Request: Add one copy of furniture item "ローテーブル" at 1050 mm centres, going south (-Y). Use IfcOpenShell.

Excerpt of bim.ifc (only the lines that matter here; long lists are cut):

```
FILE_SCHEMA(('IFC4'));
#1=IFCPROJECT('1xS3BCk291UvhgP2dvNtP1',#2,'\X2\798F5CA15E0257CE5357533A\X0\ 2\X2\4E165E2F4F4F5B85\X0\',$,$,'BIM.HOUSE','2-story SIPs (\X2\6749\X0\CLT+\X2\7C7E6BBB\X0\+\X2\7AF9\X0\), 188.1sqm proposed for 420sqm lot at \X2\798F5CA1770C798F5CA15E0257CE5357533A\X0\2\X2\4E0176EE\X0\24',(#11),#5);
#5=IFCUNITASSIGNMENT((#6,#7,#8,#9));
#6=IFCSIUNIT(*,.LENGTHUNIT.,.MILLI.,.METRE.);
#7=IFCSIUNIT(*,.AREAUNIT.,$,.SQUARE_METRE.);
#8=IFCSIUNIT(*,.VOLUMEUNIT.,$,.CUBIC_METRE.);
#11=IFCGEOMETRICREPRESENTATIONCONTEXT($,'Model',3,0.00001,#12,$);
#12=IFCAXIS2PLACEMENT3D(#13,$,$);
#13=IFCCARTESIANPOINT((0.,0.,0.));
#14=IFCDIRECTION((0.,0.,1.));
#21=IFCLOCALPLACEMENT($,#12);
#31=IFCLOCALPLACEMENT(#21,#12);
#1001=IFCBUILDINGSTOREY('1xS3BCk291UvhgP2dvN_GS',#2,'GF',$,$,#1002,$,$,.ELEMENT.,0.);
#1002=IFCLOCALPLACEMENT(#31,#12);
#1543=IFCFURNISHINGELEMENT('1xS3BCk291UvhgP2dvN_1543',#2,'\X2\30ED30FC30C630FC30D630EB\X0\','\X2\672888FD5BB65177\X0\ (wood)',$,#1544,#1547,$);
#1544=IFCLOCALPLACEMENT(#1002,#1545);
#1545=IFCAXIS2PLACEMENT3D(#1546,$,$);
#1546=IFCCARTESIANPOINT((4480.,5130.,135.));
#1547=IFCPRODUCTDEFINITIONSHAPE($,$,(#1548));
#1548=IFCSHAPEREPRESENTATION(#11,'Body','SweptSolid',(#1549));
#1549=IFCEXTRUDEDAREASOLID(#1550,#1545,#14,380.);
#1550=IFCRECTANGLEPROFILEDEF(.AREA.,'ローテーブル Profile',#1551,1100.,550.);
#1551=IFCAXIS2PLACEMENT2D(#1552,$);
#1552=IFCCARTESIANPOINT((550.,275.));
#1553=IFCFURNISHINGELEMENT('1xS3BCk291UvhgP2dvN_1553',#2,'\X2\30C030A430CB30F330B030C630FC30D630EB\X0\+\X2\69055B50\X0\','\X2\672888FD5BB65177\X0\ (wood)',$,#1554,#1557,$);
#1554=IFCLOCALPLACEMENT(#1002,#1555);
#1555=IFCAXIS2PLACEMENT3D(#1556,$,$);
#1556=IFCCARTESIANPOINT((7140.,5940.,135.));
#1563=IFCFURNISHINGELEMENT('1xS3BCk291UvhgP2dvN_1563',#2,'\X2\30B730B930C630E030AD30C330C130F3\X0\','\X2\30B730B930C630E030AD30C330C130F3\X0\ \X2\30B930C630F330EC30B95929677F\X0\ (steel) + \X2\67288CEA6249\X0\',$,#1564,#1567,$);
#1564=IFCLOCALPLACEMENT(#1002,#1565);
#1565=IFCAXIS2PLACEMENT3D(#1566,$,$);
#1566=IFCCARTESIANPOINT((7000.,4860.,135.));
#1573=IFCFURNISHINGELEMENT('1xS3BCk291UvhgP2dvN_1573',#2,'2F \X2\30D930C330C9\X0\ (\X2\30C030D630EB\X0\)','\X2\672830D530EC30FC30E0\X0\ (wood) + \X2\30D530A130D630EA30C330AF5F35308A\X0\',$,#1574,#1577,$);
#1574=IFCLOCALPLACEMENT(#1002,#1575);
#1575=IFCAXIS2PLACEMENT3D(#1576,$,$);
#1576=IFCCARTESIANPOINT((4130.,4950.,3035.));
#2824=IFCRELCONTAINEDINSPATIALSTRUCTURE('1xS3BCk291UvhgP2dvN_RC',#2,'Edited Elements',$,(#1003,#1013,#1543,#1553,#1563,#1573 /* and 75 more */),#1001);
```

```python
import numpy as np
import ifcopenshell
import ifcopenshell.api.geometry
import ifcopenshell.api.root
import ifcopenshell.util.element
import ifcopenshell.util.placement
import ifcopenshell.util.unit

model = ifcopenshell.open("bim.ifc")
unit_scale = ifcopenshell.util.unit.calculate_unit_scale(model)


def reuse_history(source, copy):
    """copy_class also copies each property set's owner history, people and application; keep the originals."""
    for rel in copy.IsDefinedBy:
        if rel.is_a("IfcRelDefinesByProperties") and (history := rel.RelatingPropertyDefinition.OwnerHistory):
            rel.RelatingPropertyDefinition.OwnerHistory = source.OwnerHistory
            ifcopenshell.util.element.remove_deep2(model, history)


source = model.by_guid("1xS3BCk291UvhgP2dvN_1543")
base = ifcopenshell.util.placement.get_local_placement(source.ObjectPlacement)
step = np.array([0.0, -1.0, 0.0]) * 1.05 / unit_scale

for i in range(1, 2):
    copy = ifcopenshell.api.root.copy_class(model, product=source)
    copy.Representation = ifcopenshell.util.element.copy_deep(
        model, source.Representation, exclude=["IfcGeometricRepresentationContext", "IfcRepresentationMap"]
    )
    reuse_history(source, copy)
    matrix = base.copy()
    matrix[:3, 3] += i * step
    print("added at", matrix[:3, 3].round(3) + 0.0)
    ifcopenshell.api.geometry.edit_object_placement(model, product=copy, matrix=matrix, is_si=False)

model.write("bim_updated.ifc")
```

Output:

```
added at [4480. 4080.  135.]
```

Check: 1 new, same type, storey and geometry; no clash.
